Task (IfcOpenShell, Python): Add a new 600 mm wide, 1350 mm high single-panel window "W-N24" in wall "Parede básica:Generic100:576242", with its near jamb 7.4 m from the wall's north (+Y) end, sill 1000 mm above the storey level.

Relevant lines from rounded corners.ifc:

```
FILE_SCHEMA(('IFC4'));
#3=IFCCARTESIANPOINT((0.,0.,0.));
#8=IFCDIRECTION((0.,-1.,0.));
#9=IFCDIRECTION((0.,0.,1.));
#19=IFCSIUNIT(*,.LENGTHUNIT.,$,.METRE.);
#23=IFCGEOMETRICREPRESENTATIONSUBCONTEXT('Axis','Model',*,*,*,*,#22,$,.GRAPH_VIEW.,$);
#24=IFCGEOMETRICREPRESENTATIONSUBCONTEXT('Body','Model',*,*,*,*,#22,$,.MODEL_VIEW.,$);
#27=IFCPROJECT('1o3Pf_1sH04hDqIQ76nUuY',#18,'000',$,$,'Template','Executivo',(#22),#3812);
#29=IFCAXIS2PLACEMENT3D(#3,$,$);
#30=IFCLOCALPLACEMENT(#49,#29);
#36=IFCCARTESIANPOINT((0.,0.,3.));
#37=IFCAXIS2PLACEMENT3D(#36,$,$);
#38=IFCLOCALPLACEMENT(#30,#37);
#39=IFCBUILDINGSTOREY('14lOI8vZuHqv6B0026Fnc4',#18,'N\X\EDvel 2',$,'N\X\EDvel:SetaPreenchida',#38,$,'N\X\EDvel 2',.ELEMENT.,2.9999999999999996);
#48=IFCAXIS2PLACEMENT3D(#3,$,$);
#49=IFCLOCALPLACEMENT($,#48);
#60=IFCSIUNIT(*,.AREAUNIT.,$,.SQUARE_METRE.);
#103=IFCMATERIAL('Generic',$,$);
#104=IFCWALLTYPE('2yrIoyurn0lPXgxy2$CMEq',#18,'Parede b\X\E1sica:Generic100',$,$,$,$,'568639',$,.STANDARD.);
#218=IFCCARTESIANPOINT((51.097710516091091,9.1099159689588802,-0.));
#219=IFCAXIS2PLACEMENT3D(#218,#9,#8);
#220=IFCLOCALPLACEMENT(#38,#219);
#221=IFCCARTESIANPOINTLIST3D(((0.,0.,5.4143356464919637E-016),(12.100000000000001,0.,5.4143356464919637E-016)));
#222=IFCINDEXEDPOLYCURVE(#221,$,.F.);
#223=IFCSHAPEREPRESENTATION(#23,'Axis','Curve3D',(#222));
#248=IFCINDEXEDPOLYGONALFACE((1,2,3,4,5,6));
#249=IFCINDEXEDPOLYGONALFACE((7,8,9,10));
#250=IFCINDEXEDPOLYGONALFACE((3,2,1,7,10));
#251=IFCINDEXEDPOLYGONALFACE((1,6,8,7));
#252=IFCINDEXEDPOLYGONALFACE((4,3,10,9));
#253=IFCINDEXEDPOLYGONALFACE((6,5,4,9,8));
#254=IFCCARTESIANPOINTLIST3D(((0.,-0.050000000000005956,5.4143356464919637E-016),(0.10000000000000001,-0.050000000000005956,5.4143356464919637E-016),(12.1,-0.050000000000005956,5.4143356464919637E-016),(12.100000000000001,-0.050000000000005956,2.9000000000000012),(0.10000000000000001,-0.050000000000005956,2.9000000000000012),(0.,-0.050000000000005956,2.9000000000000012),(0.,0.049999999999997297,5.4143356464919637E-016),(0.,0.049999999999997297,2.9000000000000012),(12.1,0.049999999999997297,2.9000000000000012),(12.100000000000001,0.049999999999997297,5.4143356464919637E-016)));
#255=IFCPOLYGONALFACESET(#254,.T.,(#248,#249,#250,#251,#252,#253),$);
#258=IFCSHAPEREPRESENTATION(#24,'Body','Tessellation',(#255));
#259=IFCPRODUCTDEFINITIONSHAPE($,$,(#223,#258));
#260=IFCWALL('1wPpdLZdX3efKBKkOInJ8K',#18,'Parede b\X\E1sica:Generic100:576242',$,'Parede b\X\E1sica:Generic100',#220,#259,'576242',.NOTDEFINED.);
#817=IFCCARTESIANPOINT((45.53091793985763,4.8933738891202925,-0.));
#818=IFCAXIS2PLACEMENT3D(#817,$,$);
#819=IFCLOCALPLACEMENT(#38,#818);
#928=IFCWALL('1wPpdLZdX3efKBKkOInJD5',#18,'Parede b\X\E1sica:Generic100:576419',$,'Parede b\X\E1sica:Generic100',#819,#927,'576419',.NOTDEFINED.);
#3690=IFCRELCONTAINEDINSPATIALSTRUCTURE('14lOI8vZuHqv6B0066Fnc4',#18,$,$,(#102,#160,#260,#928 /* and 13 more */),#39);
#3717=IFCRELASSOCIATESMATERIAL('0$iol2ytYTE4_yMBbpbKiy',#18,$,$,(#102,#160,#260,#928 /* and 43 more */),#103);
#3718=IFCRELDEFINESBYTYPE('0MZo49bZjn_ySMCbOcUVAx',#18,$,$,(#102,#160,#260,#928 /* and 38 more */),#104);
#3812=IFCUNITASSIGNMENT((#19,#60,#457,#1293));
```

```python
import numpy as np
import ifcopenshell
import ifcopenshell.api.feature
import ifcopenshell.api.geometry
import ifcopenshell.api.root
import ifcopenshell.api.spatial
import ifcopenshell.geom
import ifcopenshell.util.element
import ifcopenshell.util.placement
import ifcopenshell.util.representation
import ifcopenshell.util.shape
import ifcopenshell.util.unit

model = ifcopenshell.open("rounded corners.ifc")
unit_scale = ifcopenshell.util.unit.calculate_unit_scale(model)
settings = ifcopenshell.geom.settings()


def volume(element):
    """Net volume in cubic metres, openings subtracted."""
    shape = ifcopenshell.geom.create_shape(settings, element)
    return ifcopenshell.util.shape.get_volume(shape.geometry)


wall = model.by_guid("1wPpdLZdX3efKBKkOInJ8K")
storey = ifcopenshell.util.element.get_container(wall, ifc_class="IfcBuildingStorey")
context = ifcopenshell.util.representation.get_context(model, "Model", "Body", "MODEL_VIEW")
before = volume(wall)

width, height, from_end, sill = 0.6, 1.35, 7.4, 1  # metres

# The wall runs along its own X axis, and the end named is its -X end.
wall_shape = ifcopenshell.geom.create_shape(settings, wall)
x, y, z = ifcopenshell.util.shape.get_vertices(wall_shape.geometry).T
start = x.min() + from_end
face, thickness = float(y.min()), float(y.max() - y.min())
wall_matrix = ifcopenshell.util.placement.get_local_placement(wall.ObjectPlacement)
level = ifcopenshell.util.placement.get_local_placement(storey.ObjectPlacement)[2, 3]


def in_wall(x, y):
    """Placement at x, y metres in the wall's axes, at sill height."""
    matrix = wall_matrix.copy()
    matrix[:, 3] = wall_matrix @ np.array([x / unit_scale, y / unit_scale, 0.0, 1.0])
    matrix[2, 3] = level + sill / unit_scale
    return matrix


# Opening: a box that overshoots both wall faces by 50 mm.
opening = ifcopenshell.api.root.create_entity(model, ifc_class="IfcOpeningElement", predefined_type="OPENING")
box = ifcopenshell.api.geometry.add_wall_representation(
    model, context=context, length=width, height=height, thickness=thickness + 0.1
)
ifcopenshell.api.geometry.assign_representation(model, product=opening, representation=box)
ifcopenshell.api.geometry.edit_object_placement(model, product=opening, matrix=in_wall(start, face - 0.05), is_si=False)
ifcopenshell.api.feature.add_feature(model, feature=opening, element=wall)

window = ifcopenshell.api.root.create_entity(model, ifc_class="IfcWindow", name="W-N24", predefined_type="WINDOW")
window.OverallWidth, window.OverallHeight = width / unit_scale, height / unit_scale
window.PartitioningType = "SINGLE_PANEL"
body = ifcopenshell.api.geometry.add_window_representation(
    model,
    context=context,
    overall_width=window.OverallWidth,
    overall_height=window.OverallHeight,
    partition_type="SINGLE_PANEL",
)
ifcopenshell.api.geometry.assign_representation(model, product=window, representation=body)
ifcopenshell.api.spatial.assign_container(model, products=[window], relating_structure=storey)
ifcopenshell.api.feature.add_filling(model, opening=opening, element=window)

# Centre the window in the wall's thickness.
ifcopenshell.api.geometry.edit_object_placement(model, product=window, matrix=in_wall(start, face), is_si=False)
window_shape = ifcopenshell.geom.create_shape(settings, window)
depth = ifcopenshell.util.shape.get_vertices(window_shape.geometry)[:, 1]
offset = face + thickness / 2 - (depth.min() + depth.max()) / 2
ifcopenshell.api.geometry.edit_object_placement(model, product=window, matrix=in_wall(start, offset), is_si=False)

after = volume(wall)

print(f"wall volume {before:.3f} -> {after:.3f} m3")

model.write("rounded corners_edited.ifc")
```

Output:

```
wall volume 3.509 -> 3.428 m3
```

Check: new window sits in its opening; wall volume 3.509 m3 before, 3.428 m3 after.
